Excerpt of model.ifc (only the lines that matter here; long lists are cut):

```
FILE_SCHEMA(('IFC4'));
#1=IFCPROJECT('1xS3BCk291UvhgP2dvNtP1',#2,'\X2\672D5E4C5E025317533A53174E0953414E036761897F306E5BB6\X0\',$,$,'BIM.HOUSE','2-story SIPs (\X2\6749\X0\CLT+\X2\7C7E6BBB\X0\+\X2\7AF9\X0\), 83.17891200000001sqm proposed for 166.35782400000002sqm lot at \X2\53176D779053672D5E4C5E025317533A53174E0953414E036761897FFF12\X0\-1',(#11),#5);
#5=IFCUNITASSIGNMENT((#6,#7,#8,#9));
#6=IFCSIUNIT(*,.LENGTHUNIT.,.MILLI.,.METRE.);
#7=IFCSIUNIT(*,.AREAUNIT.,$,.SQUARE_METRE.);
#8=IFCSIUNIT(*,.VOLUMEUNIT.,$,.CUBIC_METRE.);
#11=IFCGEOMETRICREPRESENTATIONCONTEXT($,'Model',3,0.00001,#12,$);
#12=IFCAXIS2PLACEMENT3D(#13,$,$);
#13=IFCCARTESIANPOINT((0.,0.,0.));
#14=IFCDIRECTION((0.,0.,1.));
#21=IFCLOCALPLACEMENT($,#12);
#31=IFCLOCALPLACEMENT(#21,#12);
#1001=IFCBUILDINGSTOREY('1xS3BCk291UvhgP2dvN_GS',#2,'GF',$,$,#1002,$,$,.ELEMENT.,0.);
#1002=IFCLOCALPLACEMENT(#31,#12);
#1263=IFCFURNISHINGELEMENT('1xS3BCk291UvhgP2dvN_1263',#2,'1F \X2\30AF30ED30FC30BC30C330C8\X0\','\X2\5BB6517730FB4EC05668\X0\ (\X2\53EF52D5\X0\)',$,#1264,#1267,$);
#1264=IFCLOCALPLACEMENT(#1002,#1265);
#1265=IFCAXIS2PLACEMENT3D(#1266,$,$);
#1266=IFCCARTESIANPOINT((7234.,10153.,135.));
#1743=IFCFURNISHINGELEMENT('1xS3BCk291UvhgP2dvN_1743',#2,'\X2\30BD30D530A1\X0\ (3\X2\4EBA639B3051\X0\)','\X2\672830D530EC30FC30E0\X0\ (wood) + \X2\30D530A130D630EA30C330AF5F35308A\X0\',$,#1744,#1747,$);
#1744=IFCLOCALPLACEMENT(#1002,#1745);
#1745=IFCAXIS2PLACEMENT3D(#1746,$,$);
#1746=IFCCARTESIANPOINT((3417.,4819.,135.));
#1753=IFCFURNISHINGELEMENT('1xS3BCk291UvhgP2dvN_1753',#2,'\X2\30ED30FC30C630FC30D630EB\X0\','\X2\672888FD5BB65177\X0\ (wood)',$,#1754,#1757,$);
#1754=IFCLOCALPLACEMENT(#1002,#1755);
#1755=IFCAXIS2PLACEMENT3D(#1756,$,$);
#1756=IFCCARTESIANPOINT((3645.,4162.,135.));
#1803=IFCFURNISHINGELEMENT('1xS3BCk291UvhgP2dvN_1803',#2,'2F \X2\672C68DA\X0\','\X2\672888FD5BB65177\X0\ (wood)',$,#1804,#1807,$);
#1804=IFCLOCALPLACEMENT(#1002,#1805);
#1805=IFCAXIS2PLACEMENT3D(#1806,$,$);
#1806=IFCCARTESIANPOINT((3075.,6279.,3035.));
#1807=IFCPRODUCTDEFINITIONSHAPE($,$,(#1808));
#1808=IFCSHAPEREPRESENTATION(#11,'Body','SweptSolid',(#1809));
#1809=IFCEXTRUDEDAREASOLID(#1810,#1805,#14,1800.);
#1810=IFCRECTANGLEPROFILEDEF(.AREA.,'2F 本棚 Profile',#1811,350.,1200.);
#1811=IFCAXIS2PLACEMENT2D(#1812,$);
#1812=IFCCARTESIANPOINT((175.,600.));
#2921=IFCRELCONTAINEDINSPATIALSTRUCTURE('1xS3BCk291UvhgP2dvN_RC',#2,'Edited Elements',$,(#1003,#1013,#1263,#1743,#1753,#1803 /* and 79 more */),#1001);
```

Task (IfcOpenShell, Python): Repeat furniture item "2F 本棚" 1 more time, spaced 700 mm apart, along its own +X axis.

```python
import ifcopenshell
import ifcopenshell.api.geometry
import ifcopenshell.api.root
import ifcopenshell.util.element
import ifcopenshell.util.placement

model = ifcopenshell.open("model.ifc")


def reuse_history(source, copy):
    """copy_class also copies each property set's owner history, people and application; keep the originals."""
    for rel in copy.IsDefinedBy:
        if rel.is_a("IfcRelDefinesByProperties") and (history := rel.RelatingPropertyDefinition.OwnerHistory):
            rel.RelatingPropertyDefinition.OwnerHistory = source.OwnerHistory
            ifcopenshell.util.element.remove_deep2(model, history)


source = model.by_guid("1xS3BCk291UvhgP2dvN_1803")
base = ifcopenshell.util.placement.get_local_placement(source.ObjectPlacement)
step = base[:3, 0] * 700.0

for i in range(1, 2):
    copy = ifcopenshell.api.root.copy_class(model, product=source)
    copy.Representation = ifcopenshell.util.element.copy_deep(
        model, source.Representation, exclude=["IfcGeometricRepresentationContext", "IfcRepresentationMap"]
    )
    reuse_history(source, copy)
    matrix = base.copy()
    matrix[:3, 3] += i * step
    print("added at", matrix[:3, 3].round(3) + 0.0)
    ifcopenshell.api.geometry.edit_object_placement(model, product=copy, matrix=matrix, is_si=False)

model.write("model_v2.ifc")
```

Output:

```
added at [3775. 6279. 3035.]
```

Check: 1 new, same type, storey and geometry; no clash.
